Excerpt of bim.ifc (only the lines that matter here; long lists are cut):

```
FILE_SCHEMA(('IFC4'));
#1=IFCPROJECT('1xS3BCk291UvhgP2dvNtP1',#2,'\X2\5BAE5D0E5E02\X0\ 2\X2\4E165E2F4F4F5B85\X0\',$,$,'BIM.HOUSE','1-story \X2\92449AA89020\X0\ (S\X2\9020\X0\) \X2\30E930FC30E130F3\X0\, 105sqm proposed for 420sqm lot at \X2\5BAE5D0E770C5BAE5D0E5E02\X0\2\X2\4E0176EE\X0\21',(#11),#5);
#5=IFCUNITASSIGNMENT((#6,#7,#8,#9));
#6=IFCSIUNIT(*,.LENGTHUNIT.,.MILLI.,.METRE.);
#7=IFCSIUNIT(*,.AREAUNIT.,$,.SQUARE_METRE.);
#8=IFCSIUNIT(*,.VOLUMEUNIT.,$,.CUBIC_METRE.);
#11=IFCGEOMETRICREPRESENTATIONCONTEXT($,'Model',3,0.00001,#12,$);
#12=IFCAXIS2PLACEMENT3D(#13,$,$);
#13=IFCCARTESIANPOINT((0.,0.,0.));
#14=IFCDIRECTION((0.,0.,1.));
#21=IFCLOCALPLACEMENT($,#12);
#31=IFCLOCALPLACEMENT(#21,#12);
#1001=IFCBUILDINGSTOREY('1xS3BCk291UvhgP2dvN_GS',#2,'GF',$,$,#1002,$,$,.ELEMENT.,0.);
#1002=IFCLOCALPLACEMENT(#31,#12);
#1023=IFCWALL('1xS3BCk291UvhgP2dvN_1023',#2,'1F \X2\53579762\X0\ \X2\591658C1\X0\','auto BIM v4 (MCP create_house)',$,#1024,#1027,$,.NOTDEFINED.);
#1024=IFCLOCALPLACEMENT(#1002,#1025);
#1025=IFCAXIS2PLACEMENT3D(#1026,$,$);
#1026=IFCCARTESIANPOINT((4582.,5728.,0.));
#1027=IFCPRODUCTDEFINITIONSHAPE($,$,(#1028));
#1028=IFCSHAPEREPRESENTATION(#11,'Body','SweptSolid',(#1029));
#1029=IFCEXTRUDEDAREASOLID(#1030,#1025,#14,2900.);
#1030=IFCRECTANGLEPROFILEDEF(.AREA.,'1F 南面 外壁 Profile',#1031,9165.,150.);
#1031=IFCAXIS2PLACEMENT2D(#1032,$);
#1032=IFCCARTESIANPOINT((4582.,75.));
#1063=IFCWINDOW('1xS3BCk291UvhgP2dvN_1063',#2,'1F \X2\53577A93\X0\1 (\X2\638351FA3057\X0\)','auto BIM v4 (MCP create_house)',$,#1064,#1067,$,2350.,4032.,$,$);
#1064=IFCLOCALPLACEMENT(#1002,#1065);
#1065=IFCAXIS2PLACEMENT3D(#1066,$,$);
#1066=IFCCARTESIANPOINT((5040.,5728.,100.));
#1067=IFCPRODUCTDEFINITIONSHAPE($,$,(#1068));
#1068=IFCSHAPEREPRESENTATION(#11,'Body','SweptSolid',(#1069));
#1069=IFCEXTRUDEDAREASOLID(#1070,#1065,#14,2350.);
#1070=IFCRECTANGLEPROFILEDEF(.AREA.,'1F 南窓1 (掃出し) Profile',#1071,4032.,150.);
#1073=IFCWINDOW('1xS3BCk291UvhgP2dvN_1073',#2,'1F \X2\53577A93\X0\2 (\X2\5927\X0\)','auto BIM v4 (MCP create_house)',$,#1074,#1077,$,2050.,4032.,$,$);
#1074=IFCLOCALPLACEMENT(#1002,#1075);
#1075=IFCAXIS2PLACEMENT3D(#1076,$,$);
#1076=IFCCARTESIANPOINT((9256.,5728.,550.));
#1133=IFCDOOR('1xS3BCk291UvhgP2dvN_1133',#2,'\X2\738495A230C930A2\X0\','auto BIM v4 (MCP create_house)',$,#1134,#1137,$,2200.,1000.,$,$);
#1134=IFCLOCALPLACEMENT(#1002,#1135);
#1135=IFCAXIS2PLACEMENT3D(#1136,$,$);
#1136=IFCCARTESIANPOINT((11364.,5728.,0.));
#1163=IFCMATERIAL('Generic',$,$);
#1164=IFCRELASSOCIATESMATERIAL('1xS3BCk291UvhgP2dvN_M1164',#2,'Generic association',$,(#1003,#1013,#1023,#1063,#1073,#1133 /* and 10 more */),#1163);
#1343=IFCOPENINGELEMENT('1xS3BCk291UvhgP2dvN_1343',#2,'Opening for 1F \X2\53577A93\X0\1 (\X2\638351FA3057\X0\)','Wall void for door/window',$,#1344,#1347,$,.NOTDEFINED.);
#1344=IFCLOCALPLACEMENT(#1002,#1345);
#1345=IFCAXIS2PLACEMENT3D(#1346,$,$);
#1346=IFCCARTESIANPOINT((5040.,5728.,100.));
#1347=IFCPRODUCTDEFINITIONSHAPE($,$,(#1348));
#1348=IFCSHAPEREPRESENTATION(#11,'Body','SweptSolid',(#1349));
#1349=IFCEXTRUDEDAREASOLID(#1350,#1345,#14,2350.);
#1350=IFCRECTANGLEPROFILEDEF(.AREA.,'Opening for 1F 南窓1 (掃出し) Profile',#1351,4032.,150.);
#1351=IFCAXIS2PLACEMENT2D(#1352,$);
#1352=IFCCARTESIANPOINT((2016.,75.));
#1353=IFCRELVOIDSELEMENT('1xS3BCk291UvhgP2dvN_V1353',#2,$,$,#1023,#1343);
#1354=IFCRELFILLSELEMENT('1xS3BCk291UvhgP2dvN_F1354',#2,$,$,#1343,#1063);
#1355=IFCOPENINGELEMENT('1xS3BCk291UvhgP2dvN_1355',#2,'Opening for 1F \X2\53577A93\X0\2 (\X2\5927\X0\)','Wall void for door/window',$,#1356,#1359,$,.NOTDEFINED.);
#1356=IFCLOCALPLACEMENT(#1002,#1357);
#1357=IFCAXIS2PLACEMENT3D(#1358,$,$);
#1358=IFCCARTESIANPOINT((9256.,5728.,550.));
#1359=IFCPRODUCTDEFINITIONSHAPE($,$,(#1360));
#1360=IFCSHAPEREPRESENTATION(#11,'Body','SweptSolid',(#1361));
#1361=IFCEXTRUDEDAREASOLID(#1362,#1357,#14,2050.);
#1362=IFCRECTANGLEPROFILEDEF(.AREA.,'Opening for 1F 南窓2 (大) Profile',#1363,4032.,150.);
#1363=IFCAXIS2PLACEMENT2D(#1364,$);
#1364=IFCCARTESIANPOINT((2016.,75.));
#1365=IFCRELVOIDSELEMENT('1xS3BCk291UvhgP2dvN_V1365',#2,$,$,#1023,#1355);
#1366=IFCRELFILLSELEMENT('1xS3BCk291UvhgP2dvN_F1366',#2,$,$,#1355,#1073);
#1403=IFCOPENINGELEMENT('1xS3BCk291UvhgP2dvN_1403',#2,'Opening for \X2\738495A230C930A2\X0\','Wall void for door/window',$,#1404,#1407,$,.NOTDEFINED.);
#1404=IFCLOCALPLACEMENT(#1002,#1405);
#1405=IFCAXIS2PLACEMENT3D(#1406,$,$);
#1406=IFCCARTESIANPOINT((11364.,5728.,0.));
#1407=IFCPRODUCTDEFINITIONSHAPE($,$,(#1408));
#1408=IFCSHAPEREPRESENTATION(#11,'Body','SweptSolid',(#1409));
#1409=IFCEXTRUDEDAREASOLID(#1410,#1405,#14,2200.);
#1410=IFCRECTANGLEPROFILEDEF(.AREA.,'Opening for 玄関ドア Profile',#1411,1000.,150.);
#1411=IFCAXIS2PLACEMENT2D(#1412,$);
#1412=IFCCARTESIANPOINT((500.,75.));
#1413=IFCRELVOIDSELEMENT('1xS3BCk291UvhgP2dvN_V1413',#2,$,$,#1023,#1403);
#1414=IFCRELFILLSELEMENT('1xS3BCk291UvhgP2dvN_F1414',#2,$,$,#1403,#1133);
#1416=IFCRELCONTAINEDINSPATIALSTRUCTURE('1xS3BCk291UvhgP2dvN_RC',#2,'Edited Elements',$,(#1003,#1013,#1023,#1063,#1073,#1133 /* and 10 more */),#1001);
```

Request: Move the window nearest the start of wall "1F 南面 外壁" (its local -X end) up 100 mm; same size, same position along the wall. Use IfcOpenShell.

```python
import numpy as np
import ifcopenshell
import ifcopenshell.api.geometry
import ifcopenshell.util.placement
import ifcopenshell.util.unit

model = ifcopenshell.open("bim.ifc")
unit_scale = ifcopenshell.util.unit.calculate_unit_scale(model)

window = model.by_guid("1xS3BCk291UvhgP2dvN_1063")
opening = window.FillsVoids[0].RelatingOpeningElement
dz = 0.1 / unit_scale

shift = np.array([0.0, 0.0, dz])
# The window is not placed relative to its opening, so move both.
for product in (opening, window):
    matrix = ifcopenshell.util.placement.get_local_placement(product.ObjectPlacement)
    matrix[:3, 3] += shift
    ifcopenshell.api.geometry.edit_object_placement(model, product=product, matrix=matrix, is_si=False)

print(f"moved by {dz * unit_scale:+.3f} m")

model.write("bim_updated.ifc")
```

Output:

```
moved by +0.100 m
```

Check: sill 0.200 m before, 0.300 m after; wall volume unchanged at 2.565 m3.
